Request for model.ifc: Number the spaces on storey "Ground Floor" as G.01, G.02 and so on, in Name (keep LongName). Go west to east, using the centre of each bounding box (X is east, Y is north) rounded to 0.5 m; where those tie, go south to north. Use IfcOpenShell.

First a look at what the model holds.

```python
import ifcopenshell
import ifcopenshell.util.element
import ifcopenshell.util.placement

model = ifcopenshell.open("model.ifc")
print(model.schema)
storey = next(s for s in model.by_type("IfcBuildingStorey") if s.Name == "Ground Floor")
spaces = [e for e in ifcopenshell.util.element.get_decomposition(storey) if e.is_a("IfcSpace")]
for e in sorted(spaces, key=lambda e: e.id()):
    origin = ifcopenshell.util.placement.get_local_placement(e.ObjectPlacement)[:3, 3]
    print(e.id(), e.Name, e.LongName, origin.round(2) + 0.0, sep=" | ")
```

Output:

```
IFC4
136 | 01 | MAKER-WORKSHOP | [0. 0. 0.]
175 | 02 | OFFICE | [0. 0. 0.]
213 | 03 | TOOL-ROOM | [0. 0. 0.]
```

```python
import ifcopenshell
import ifcopenshell.geom
import ifcopenshell.util.element
import ifcopenshell.util.shape

model = ifcopenshell.open("model.ifc")
settings = ifcopenshell.geom.settings()
settings.set("use-world-coords", True)


def centre(element):
    shape = ifcopenshell.geom.create_shape(settings, element)
    return ifcopenshell.util.shape.get_bbox_centroid(shape.geometry)


storey = next(s for s in model.by_type("IfcBuildingStorey") if s.Name == "Ground Floor")
spaces = [e for e in ifcopenshell.util.element.get_decomposition(storey) if e.is_a("IfcSpace")]

# Insertion points can sit at a corner or the storey origin, so sort by the geometry (in metres).
centres = {e: centre(e) for e in spaces}
spaces.sort(key=lambda e: (round(centres[e][0] / 0.5), centres[e][1]))

for i, e in enumerate(spaces, start=1):
    number = f"G.{i:02d}"
    e.Name = number
    print(e.id(), number)

model.write("model_rev.ifc")
```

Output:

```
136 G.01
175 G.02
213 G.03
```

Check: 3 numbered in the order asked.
